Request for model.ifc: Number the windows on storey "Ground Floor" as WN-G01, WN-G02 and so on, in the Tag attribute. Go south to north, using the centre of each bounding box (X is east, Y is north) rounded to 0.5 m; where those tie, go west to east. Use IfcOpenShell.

First a look at what the model holds.

```python
import ifcopenshell
import ifcopenshell.util.element
import ifcopenshell.util.placement

model = ifcopenshell.open("model.ifc")
print(model.schema)
storey = next(s for s in model.by_type("IfcBuildingStorey") if s.Name == "Ground Floor")
windows = [e for e in ifcopenshell.util.element.get_decomposition(storey) if e.is_a("IfcWindow")]
for e in sorted(windows, key=lambda e: e.id()):
    origin = ifcopenshell.util.placement.get_local_placement(e.ObjectPlacement)[:3, 3]
    print(e.id(), e.Tag, e.Name, origin.round(2) + 0.0, sep=" | ")
```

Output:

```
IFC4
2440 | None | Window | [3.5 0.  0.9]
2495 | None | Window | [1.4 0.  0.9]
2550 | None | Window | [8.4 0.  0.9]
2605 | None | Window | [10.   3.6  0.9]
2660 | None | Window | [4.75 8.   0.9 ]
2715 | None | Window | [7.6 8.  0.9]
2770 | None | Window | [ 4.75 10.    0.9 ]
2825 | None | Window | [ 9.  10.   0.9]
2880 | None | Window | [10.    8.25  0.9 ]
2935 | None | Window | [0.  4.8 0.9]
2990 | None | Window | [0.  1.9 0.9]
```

```python
import ifcopenshell
import ifcopenshell.geom
import ifcopenshell.util.element
import ifcopenshell.util.shape

model = ifcopenshell.open("model.ifc")
settings = ifcopenshell.geom.settings()
settings.set("use-world-coords", True)


def centre(element):
    shape = ifcopenshell.geom.create_shape(settings, element)
    return ifcopenshell.util.shape.get_bbox_centroid(shape.geometry)


storey = next(s for s in model.by_type("IfcBuildingStorey") if s.Name == "Ground Floor")
windows = [e for e in ifcopenshell.util.element.get_decomposition(storey) if e.is_a("IfcWindow")]

# Insertion points can sit at a corner or the storey origin, so sort by the geometry (in metres).
centres = {e: centre(e) for e in windows}
windows.sort(key=lambda e: (round(centres[e][1] / 0.5), centres[e][0]))

for i, e in enumerate(windows, start=1):
    number = f"WN-G{i:02d}"
    e.Tag = number
    print(e.id(), number)

model.write("model_edited.ifc")
```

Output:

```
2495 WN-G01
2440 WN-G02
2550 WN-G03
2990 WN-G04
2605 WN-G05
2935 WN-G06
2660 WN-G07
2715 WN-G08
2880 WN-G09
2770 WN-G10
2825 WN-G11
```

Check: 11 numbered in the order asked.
